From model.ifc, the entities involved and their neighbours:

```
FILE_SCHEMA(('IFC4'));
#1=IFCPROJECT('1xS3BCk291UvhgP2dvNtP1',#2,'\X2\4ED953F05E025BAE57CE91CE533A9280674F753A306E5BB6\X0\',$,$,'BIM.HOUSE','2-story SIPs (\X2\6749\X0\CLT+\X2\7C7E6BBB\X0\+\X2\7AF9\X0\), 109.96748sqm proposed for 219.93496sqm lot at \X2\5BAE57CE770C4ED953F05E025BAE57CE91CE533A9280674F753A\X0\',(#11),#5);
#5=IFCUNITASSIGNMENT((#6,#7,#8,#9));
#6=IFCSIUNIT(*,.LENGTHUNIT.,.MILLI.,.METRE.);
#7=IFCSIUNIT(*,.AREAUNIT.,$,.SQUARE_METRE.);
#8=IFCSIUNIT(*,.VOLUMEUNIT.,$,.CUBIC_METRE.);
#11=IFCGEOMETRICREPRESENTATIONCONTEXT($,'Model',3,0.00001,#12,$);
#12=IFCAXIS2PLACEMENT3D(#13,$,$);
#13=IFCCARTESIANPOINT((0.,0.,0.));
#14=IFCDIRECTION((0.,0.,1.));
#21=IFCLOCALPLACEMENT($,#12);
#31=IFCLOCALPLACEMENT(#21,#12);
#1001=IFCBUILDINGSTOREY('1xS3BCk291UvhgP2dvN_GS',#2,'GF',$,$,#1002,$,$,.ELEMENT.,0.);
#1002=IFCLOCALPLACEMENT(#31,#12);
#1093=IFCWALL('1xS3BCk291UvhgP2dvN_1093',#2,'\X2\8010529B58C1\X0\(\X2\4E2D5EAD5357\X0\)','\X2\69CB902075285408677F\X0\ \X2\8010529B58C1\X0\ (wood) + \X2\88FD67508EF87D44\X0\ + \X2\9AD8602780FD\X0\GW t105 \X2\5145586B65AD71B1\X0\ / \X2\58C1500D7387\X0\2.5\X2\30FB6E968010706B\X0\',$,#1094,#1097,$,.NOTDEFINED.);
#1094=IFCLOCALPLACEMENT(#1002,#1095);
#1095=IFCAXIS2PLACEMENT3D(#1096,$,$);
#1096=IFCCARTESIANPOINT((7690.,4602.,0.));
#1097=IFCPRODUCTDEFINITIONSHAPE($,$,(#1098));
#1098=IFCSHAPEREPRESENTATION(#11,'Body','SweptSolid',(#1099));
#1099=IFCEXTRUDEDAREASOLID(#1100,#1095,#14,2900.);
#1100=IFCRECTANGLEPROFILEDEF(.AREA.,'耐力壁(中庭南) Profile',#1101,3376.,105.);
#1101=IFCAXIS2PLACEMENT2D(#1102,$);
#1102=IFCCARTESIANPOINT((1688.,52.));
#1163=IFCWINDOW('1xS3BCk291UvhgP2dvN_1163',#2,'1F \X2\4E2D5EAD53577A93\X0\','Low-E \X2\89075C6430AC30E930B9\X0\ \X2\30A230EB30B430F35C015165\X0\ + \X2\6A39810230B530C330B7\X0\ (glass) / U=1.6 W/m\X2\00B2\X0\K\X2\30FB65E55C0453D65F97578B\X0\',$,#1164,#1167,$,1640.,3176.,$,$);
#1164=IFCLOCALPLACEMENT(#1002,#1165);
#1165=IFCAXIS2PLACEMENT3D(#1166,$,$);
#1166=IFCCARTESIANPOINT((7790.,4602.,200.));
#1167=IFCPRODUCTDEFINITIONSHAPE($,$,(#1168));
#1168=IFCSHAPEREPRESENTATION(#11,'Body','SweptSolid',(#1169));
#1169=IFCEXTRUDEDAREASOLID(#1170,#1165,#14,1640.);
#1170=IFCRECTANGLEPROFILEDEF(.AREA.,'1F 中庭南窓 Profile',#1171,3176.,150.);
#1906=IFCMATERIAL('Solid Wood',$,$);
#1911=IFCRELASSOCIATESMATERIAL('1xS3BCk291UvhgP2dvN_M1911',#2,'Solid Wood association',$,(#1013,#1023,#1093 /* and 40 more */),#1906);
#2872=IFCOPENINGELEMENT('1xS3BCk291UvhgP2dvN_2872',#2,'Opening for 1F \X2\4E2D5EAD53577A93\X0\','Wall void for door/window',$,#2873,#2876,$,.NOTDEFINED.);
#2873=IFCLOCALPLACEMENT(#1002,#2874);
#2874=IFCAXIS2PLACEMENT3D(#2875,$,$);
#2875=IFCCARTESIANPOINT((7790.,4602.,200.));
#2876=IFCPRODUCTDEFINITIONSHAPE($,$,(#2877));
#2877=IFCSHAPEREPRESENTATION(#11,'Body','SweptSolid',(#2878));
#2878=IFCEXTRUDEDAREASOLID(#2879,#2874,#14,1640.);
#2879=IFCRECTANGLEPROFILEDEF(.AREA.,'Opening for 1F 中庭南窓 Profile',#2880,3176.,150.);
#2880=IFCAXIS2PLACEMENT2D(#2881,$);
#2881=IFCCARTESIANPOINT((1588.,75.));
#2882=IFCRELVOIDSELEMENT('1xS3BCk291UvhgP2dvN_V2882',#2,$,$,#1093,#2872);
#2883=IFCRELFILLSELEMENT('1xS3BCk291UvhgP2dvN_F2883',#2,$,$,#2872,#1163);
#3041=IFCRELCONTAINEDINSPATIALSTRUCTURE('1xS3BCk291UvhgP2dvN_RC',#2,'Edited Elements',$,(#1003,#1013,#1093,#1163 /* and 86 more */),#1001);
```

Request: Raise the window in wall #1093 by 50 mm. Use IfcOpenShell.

```python
import numpy as np
import ifcopenshell
import ifcopenshell.api.geometry
import ifcopenshell.util.placement
import ifcopenshell.util.unit

model = ifcopenshell.open("model.ifc")
unit_scale = ifcopenshell.util.unit.calculate_unit_scale(model)

window = model.by_guid("1xS3BCk291UvhgP2dvN_1163")
opening = window.FillsVoids[0].RelatingOpeningElement
dz = 0.05 / unit_scale

shift = np.array([0.0, 0.0, dz])
# The window is not placed relative to its opening, so move both.
for product in (opening, window):
    matrix = ifcopenshell.util.placement.get_local_placement(product.ObjectPlacement)
    matrix[:3, 3] += shift
    ifcopenshell.api.geometry.edit_object_placement(model, product=product, matrix=matrix, is_si=False)

print(f"moved by {dz * unit_scale:+.3f} m")

model.write("model_rev.ifc")
```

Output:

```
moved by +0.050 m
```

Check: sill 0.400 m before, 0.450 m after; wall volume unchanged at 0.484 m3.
